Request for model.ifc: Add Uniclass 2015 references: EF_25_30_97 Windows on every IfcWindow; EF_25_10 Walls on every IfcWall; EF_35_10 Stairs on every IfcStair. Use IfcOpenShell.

First a look at what the model holds.

```python
import ifcopenshell

model = ifcopenshell.open("model.ifc")
print(model.schema)
print("classifications:", [c.Name for c in model.by_type("IfcClassification")])
for ifc_class in ("IfcDoor", "IfcRoof", "IfcStair", "IfcWall", "IfcWindow"):
    print(ifc_class, len(model.by_type(ifc_class)))
```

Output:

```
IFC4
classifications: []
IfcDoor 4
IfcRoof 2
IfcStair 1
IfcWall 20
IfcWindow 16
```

```python
import ifcopenshell
import ifcopenshell.api.classification

model = ifcopenshell.open("model.ifc")

system = ifcopenshell.api.classification.add_classification(model, classification="Uniclass 2015")

codes = {
    "IfcWindow": ("EF_25_30_97", "Windows"),
    "IfcWall": ("EF_25_10", "Walls"),
    "IfcStair": ("EF_35_10", "Stairs"),
}
for ifc_class, (code, name) in codes.items():
    products = model.by_type(ifc_class)
    ifcopenshell.api.classification.add_reference(
        model, products=products, classification=system, identification=code, name=name
    )
    print(code, len(products))

model.write("model_rev.ifc")
```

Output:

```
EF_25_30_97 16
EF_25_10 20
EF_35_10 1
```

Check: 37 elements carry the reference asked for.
